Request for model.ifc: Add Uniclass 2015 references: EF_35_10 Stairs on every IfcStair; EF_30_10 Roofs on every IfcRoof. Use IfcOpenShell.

First a look at what the model holds.

```python
import ifcopenshell

model = ifcopenshell.open("model.ifc")
print(model.schema)
print("classifications:", [c.Name for c in model.by_type("IfcClassification")])
for ifc_class in ("IfcDoor", "IfcRoof", "IfcStair", "IfcWall", "IfcWindow"):
    print(ifc_class, len(model.by_type(ifc_class)))
```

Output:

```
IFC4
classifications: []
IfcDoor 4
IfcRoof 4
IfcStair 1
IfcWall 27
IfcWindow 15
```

```python
import ifcopenshell
import ifcopenshell.api.classification

model = ifcopenshell.open("model.ifc")

system = ifcopenshell.api.classification.add_classification(model, classification="Uniclass 2015")

codes = {
    "IfcStair": ("EF_35_10", "Stairs"),
    "IfcRoof": ("EF_30_10", "Roofs"),
}
for ifc_class, (code, name) in codes.items():
    products = model.by_type(ifc_class)
    ifcopenshell.api.classification.add_reference(
        model, products=products, classification=system, identification=code, name=name
    )
    print(code, len(products))

model.write("model_edited.ifc")
```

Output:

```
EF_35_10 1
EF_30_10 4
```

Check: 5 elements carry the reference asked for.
